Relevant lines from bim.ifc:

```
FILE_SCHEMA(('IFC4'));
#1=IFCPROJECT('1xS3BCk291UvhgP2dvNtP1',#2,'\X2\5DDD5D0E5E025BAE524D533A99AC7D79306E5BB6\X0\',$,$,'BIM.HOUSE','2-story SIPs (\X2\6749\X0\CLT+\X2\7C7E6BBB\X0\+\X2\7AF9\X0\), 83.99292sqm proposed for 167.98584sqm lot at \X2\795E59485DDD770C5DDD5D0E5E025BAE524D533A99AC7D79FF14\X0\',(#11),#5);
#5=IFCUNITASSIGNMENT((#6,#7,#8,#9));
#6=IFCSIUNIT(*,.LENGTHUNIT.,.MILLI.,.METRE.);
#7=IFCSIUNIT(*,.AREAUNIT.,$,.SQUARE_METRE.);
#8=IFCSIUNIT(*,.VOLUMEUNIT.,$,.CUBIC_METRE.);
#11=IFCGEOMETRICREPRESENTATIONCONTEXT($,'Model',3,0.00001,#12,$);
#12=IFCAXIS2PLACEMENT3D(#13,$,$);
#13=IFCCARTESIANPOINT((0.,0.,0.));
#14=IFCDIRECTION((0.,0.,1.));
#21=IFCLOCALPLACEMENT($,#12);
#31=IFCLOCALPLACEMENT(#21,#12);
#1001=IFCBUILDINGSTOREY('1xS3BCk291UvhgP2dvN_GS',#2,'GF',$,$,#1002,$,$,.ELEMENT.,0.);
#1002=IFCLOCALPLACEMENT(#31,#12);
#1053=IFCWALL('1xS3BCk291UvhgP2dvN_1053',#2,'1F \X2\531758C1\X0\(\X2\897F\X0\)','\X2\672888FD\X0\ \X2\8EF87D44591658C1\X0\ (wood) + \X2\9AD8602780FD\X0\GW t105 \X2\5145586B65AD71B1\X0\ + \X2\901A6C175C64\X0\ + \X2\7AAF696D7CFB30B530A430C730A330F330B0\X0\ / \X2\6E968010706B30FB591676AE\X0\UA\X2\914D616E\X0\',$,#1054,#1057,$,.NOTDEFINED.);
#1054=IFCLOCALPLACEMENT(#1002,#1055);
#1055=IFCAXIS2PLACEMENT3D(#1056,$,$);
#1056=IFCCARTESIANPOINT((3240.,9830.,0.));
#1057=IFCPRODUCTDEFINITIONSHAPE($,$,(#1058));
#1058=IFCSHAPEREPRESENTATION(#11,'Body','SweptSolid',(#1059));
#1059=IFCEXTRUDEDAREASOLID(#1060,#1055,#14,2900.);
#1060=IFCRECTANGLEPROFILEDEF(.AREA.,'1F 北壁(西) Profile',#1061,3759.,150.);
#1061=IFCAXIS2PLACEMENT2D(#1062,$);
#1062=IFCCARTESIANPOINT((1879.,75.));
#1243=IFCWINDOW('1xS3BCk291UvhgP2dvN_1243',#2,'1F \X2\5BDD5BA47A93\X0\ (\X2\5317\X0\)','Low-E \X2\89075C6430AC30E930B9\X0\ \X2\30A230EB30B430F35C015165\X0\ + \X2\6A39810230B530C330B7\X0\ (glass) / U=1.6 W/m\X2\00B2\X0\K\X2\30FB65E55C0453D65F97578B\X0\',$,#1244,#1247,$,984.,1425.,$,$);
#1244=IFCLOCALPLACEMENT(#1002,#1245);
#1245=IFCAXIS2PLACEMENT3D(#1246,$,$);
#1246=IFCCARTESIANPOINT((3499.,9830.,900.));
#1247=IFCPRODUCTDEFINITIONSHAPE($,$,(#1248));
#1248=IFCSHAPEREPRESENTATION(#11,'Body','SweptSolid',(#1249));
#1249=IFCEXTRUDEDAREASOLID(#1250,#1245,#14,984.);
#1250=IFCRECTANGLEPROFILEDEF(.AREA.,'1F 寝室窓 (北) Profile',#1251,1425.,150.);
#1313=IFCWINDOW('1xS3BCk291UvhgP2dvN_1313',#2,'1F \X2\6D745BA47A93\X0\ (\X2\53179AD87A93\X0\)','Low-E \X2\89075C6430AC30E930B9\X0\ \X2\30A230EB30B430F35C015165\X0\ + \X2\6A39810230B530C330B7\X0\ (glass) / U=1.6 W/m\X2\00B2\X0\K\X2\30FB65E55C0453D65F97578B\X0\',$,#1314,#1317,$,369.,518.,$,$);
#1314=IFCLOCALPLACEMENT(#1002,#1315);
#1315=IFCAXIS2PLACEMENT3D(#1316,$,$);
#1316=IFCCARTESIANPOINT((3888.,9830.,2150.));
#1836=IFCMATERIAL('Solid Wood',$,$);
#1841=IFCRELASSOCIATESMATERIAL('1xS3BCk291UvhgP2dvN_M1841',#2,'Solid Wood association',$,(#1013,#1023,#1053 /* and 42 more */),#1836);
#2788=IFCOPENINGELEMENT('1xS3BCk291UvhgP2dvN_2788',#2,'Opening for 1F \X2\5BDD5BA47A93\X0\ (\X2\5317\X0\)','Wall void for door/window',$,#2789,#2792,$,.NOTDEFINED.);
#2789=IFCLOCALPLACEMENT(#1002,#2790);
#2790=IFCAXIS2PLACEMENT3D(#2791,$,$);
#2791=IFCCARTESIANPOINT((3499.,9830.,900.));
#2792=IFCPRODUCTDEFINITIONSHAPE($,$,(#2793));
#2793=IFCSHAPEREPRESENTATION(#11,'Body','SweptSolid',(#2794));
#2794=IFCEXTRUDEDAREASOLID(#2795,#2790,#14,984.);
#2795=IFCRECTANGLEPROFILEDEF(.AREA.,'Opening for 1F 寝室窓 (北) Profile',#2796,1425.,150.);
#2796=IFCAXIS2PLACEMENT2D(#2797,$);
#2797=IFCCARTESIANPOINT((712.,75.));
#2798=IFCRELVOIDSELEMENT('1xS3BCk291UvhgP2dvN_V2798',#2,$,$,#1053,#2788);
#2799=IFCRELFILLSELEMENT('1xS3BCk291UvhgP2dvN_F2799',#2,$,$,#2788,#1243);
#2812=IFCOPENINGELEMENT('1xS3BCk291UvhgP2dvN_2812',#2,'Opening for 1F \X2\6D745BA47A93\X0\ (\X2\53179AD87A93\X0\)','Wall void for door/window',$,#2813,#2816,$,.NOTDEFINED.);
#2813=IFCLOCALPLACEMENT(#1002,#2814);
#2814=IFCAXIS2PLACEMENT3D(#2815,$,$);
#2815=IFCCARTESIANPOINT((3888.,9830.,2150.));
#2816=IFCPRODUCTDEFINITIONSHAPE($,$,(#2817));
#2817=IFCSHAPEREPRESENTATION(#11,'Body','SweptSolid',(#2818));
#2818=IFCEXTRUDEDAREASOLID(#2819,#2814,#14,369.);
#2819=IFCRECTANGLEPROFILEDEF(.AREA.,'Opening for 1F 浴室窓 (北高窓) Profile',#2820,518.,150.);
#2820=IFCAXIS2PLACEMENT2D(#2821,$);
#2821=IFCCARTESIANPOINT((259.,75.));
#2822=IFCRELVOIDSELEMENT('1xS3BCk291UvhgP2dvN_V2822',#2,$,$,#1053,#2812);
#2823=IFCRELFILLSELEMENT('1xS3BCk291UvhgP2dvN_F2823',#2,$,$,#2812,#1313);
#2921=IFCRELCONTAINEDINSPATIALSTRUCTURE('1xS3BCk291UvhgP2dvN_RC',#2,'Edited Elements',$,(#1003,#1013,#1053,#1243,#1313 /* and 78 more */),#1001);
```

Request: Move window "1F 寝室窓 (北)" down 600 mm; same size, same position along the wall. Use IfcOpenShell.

```python
import numpy as np
import ifcopenshell
import ifcopenshell.api.geometry
import ifcopenshell.util.placement
import ifcopenshell.util.unit

model = ifcopenshell.open("bim.ifc")
unit_scale = ifcopenshell.util.unit.calculate_unit_scale(model)

window = model.by_id(1243)
opening = window.FillsVoids[0].RelatingOpeningElement
dz = -0.6 / unit_scale

shift = np.array([0.0, 0.0, dz])
# The window is not placed relative to its opening, so move both.
for product in (opening, window):
    matrix = ifcopenshell.util.placement.get_local_placement(product.ObjectPlacement)
    matrix[:3, 3] += shift
    ifcopenshell.api.geometry.edit_object_placement(model, product=product, matrix=matrix, is_si=False)

print(f"moved by {dz * unit_scale:+.3f} m")

model.write("bim_updated.ifc")
```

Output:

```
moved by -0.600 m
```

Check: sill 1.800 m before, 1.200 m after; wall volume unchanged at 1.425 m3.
